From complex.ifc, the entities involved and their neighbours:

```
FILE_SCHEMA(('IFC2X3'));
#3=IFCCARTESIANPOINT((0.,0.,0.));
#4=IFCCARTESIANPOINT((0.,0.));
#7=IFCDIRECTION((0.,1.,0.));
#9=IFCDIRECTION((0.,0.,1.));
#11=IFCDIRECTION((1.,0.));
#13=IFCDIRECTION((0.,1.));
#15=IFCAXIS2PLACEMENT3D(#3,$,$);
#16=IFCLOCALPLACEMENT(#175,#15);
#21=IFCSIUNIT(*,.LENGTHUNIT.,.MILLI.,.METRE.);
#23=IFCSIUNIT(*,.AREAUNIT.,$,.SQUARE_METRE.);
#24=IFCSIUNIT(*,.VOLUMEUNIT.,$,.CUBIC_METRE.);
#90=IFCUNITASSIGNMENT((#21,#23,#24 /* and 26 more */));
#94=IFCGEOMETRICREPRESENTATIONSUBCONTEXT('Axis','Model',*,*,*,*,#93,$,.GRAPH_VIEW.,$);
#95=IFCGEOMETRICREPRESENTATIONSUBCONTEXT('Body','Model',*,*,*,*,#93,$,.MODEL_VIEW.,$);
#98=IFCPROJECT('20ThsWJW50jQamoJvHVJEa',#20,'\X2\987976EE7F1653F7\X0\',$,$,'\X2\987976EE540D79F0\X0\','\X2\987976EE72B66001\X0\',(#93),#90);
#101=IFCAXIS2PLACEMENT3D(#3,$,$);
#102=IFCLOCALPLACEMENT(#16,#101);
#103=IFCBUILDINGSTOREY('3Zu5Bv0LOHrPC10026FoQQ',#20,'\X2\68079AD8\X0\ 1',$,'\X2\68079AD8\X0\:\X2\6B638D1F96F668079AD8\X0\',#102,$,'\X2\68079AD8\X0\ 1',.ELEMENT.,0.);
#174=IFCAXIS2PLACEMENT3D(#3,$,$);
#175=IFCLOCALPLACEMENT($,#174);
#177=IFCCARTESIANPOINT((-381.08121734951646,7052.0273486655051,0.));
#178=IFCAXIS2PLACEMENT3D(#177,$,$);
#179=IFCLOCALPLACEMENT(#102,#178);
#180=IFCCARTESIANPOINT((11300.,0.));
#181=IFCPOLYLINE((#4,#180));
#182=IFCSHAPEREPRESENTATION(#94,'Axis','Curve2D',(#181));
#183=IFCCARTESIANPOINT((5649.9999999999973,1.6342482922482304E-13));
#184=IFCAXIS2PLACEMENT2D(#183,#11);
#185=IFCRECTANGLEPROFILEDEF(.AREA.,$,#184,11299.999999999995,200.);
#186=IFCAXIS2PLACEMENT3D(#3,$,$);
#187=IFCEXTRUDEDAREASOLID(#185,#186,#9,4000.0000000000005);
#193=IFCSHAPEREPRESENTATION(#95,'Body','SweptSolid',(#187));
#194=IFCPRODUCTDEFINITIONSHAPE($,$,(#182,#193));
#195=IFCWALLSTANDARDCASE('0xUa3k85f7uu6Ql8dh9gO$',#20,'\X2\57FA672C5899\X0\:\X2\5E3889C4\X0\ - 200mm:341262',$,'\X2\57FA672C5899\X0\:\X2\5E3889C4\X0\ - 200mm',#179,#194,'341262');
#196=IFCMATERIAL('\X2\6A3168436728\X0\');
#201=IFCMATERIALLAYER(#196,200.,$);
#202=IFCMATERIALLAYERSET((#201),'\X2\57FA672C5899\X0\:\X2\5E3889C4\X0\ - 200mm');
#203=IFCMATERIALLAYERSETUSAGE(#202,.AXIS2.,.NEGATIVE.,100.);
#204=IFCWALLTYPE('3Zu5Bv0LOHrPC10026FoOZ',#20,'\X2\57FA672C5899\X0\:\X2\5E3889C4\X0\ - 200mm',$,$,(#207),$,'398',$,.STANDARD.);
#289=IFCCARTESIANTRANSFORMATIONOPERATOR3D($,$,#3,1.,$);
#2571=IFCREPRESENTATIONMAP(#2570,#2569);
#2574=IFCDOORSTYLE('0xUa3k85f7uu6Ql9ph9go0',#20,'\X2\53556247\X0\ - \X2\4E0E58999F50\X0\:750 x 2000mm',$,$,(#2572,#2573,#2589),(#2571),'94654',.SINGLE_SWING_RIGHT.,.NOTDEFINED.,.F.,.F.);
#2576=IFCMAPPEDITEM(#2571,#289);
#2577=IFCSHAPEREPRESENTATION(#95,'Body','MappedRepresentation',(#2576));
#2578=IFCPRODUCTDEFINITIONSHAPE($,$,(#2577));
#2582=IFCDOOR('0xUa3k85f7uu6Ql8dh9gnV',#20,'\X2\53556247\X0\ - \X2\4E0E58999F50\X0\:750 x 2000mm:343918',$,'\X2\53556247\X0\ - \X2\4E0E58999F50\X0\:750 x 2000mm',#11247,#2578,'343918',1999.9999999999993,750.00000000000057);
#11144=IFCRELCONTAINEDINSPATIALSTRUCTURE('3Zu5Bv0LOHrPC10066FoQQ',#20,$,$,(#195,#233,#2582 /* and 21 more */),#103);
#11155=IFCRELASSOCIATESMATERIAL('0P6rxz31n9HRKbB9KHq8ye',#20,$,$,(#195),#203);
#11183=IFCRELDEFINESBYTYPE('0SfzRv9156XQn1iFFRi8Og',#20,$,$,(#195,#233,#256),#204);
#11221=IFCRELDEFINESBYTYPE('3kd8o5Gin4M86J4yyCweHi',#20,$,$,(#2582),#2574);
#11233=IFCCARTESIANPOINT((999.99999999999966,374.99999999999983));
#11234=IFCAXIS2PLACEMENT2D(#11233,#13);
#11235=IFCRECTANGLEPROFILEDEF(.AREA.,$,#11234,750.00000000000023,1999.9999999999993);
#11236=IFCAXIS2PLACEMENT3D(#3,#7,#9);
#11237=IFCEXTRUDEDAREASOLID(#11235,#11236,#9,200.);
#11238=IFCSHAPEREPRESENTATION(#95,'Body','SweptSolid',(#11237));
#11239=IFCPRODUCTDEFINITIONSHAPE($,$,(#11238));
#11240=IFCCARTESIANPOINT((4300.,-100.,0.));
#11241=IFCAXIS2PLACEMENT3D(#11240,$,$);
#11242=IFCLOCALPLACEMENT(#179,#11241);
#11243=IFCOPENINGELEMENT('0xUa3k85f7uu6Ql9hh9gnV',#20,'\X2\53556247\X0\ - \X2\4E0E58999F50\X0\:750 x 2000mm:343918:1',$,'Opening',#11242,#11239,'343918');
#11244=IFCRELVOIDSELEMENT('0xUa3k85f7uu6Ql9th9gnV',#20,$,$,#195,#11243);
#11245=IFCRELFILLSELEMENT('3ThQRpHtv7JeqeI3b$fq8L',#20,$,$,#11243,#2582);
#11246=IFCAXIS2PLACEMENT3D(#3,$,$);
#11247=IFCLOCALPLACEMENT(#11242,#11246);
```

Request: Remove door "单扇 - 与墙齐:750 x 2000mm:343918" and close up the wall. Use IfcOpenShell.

```python
import ifcopenshell
import ifcopenshell.api.feature
import ifcopenshell.api.root
import ifcopenshell.geom
import ifcopenshell.util.shape

model = ifcopenshell.open("complex.ifc")
settings = ifcopenshell.geom.settings()


def volume(element):
    """Net volume in cubic metres, openings subtracted."""
    shape = ifcopenshell.geom.create_shape(settings, element)
    return ifcopenshell.util.shape.get_volume(shape.geometry)


door = model.by_id(2582)
opening = door.FillsVoids[0].RelatingOpeningElement
wall = opening.VoidsElements[0].RelatingBuildingElement
before = volume(wall)

ifcopenshell.api.root.remove_product(model, product=door)
ifcopenshell.api.feature.remove_feature(model, feature=opening)

after = volume(wall)

print(f"wall volume {before:.3f} -> {after:.3f} m3")

model.write("complex_edited.ifc")
```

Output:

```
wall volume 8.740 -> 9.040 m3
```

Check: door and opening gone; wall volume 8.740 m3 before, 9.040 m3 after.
